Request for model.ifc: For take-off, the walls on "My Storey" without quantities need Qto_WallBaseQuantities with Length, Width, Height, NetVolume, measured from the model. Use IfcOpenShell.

First a look at what the model holds.

```python
import ifcopenshell
import ifcopenshell.util.element
import ifcopenshell.util.unit

model = ifcopenshell.open("model.ifc")
print(model.schema)
for unit_type in ("LENGTHUNIT", "AREAUNIT", "VOLUMEUNIT"):
    print(unit_type, ifcopenshell.util.unit.calculate_unit_scale(model, unit_type))
storey = next(s for s in model.by_type("IfcBuildingStorey") if s.Name == "My Storey")
walls = [e for e in ifcopenshell.util.element.get_decomposition(storey) if e.is_a("IfcWall")]
for e in sorted(walls, key=lambda e: e.id()):
    print(e.id(), e.is_a(), e.Name, list(ifcopenshell.util.element.get_psets(e, qtos_only=True)), sep=" | ")
```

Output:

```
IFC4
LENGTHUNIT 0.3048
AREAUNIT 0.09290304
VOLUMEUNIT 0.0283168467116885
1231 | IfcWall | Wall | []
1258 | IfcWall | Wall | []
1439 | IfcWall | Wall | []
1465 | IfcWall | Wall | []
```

```python
import ifcopenshell
import ifcopenshell.api.pset
import ifcopenshell.geom
import ifcopenshell.util.element
import ifcopenshell.util.shape
import ifcopenshell.util.unit

model = ifcopenshell.open("model.ifc")
unit_scale = ifcopenshell.util.unit.calculate_unit_scale(model)
volume_scale = ifcopenshell.util.unit.calculate_unit_scale(model, "VOLUMEUNIT")
settings = ifcopenshell.geom.settings()

storey = next(s for s in model.by_type("IfcBuildingStorey") if s.Name == "My Storey")
walls = [e for e in ifcopenshell.util.element.get_decomposition(storey) if e.is_a("IfcWall")]

for e in sorted(walls, key=lambda e: e.id()):
    if ifcopenshell.util.element.get_psets(e, qtos_only=True, should_inherit=False):
        continue
    # Geometry comes back in metres, in the element's own axes.
    shape = ifcopenshell.geom.create_shape(settings, e)
    values = {
        "Length": ifcopenshell.util.shape.get_x(shape.geometry) / unit_scale,
        "Width": ifcopenshell.util.shape.get_y(shape.geometry) / unit_scale,
        "Height": ifcopenshell.util.shape.get_z(shape.geometry) / unit_scale,
        "NetVolume": ifcopenshell.util.shape.get_volume(shape.geometry) / volume_scale,
    }
    qto = ifcopenshell.api.pset.add_qto(model, product=e, name="Qto_WallBaseQuantities")
    ifcopenshell.api.pset.edit_qto(model, qto=qto, properties=values)
    print(e.id(), {k: round(v, 3) for k, v in values.items()})

model.write("model-out.ifc")
```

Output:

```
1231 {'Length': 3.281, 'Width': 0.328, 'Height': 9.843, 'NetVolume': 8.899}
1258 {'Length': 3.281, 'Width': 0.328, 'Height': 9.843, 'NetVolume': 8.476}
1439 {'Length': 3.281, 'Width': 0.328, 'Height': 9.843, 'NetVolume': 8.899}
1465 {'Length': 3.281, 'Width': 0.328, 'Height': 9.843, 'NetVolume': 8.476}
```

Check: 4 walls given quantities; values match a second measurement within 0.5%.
